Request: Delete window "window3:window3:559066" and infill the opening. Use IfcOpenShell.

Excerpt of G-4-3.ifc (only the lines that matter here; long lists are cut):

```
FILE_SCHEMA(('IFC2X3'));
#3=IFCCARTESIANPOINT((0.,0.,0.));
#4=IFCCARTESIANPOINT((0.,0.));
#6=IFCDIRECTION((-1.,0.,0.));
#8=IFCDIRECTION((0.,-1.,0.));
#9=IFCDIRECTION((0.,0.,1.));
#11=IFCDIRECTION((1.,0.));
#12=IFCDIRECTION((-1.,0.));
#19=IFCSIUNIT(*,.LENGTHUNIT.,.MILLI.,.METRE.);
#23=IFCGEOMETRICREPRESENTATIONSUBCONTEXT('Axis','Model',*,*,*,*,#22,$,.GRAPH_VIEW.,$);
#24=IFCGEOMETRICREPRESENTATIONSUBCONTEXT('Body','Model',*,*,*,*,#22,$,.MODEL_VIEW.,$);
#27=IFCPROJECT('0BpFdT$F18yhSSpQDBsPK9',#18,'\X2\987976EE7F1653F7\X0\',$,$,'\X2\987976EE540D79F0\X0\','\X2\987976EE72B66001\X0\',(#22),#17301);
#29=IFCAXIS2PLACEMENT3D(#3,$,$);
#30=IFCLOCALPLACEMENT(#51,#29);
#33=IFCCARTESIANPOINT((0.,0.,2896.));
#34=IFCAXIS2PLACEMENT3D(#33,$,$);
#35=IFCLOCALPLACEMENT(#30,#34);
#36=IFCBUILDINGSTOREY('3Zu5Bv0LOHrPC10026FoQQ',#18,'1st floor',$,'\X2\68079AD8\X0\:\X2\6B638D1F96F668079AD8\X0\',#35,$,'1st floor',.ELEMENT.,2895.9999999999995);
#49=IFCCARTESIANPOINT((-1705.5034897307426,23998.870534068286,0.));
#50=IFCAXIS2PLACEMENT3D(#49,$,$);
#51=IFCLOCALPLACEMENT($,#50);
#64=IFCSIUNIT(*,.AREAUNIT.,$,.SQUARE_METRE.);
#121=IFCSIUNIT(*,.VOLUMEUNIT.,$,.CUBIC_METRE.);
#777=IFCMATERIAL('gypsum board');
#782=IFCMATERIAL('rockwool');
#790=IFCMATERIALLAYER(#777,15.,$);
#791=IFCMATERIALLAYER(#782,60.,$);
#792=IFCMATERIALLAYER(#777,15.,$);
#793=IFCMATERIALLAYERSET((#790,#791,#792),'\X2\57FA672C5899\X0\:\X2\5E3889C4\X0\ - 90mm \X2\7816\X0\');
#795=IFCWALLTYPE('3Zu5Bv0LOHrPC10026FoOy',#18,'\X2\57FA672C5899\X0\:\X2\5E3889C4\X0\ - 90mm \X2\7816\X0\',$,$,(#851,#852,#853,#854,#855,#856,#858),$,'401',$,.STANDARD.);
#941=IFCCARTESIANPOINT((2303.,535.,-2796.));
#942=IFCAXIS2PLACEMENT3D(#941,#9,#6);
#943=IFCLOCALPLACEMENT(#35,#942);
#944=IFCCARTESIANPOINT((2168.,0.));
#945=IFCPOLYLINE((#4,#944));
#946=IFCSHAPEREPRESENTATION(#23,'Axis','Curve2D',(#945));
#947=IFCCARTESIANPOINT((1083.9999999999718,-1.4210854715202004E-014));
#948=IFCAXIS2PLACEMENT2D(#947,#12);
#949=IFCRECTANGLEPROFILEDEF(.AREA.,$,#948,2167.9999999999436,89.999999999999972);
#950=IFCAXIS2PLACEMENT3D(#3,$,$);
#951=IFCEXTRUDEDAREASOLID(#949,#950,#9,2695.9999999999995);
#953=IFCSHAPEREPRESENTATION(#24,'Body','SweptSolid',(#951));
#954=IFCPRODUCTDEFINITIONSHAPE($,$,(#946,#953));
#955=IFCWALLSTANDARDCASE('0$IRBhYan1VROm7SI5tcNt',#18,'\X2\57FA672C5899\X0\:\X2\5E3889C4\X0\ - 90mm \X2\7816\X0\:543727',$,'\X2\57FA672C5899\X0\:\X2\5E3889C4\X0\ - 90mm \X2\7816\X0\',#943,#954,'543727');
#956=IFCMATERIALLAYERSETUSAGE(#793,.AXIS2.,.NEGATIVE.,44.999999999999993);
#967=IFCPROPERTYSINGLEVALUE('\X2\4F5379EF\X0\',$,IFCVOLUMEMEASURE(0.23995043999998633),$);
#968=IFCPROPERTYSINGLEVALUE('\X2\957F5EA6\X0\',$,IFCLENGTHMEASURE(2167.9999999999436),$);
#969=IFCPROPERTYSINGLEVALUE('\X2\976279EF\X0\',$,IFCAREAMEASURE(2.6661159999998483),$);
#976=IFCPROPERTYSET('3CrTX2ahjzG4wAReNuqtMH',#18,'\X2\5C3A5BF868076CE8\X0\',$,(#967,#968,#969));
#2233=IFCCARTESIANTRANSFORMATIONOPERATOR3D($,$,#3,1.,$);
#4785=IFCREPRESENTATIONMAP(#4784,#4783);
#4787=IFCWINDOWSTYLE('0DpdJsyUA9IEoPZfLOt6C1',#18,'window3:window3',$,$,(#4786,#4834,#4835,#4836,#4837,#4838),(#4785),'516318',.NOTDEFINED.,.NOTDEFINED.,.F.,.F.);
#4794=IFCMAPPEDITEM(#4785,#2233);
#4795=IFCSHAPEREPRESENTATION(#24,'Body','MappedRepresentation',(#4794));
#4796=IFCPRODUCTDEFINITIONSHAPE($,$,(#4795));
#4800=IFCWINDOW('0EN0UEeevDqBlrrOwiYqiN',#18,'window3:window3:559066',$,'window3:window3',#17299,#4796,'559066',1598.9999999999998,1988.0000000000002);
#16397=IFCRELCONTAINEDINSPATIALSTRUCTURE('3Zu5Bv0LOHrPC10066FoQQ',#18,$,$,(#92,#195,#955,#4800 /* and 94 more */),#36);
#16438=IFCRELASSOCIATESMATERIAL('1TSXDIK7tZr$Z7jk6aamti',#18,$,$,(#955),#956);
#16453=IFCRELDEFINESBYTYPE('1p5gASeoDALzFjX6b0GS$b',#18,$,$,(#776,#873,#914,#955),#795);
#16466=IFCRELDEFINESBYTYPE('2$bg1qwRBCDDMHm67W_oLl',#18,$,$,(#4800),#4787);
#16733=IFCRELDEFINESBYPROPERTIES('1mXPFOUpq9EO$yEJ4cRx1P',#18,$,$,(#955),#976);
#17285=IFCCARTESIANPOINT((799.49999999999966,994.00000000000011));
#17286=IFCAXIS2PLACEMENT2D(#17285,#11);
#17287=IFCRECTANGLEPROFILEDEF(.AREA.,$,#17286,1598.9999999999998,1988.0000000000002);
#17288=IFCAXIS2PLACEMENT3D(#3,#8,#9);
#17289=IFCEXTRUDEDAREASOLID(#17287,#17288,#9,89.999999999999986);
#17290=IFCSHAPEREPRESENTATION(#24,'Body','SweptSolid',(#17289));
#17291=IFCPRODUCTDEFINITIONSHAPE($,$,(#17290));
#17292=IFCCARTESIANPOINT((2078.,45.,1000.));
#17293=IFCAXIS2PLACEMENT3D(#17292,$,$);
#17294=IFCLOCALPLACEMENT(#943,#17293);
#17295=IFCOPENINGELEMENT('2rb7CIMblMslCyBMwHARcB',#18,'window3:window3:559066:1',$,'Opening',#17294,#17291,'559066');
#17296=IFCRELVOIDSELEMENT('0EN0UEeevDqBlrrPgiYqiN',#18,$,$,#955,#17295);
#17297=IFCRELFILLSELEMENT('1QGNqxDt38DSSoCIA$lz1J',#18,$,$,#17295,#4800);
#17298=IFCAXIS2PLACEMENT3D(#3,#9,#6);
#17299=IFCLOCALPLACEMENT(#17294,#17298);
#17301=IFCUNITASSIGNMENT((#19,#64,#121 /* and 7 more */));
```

```python
import ifcopenshell
import ifcopenshell.api.feature
import ifcopenshell.api.pset
import ifcopenshell.api.root
import ifcopenshell.geom
import ifcopenshell.util.element
import ifcopenshell.util.shape
import ifcopenshell.util.unit

model = ifcopenshell.open("G-4-3.ifc")
area_scale = ifcopenshell.util.unit.calculate_unit_scale(model, "AREAUNIT")
volume_scale = ifcopenshell.util.unit.calculate_unit_scale(model, "VOLUMEUNIT")
settings = ifcopenshell.geom.settings()


def volume(element):
    """Net volume in cubic metres, openings subtracted."""
    shape = ifcopenshell.geom.create_shape(settings, element)
    return ifcopenshell.util.shape.get_volume(shape.geometry)


window = model.by_guid("0EN0UEeevDqBlrrOwiYqiN")
opening = window.FillsVoids[0].RelatingOpeningElement
wall = opening.VoidsElements[0].RelatingBuildingElement
before = volume(wall)

ifcopenshell.api.root.remove_product(model, product=window)
ifcopenshell.api.feature.remove_feature(model, feature=opening)

after = volume(wall)
thickness = 0.09  # wall thickness in metres

# Update the wall's stored quantities.
pset = model.by_id(ifcopenshell.util.element.get_pset(wall, "尺寸标注", should_inherit=False)["id"])
ifcopenshell.api.pset.edit_pset(model, pset=pset, properties={
    "体积": model.create_entity("IfcVolumeMeasure", after / volume_scale),
    "面积": model.create_entity("IfcAreaMeasure", after / thickness / area_scale),
})

print(f"wall volume {before:.3f} -> {after:.3f} m3")

model.write("G-4-3_rev.ifc")
```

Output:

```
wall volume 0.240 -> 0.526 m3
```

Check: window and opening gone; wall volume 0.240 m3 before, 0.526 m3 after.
